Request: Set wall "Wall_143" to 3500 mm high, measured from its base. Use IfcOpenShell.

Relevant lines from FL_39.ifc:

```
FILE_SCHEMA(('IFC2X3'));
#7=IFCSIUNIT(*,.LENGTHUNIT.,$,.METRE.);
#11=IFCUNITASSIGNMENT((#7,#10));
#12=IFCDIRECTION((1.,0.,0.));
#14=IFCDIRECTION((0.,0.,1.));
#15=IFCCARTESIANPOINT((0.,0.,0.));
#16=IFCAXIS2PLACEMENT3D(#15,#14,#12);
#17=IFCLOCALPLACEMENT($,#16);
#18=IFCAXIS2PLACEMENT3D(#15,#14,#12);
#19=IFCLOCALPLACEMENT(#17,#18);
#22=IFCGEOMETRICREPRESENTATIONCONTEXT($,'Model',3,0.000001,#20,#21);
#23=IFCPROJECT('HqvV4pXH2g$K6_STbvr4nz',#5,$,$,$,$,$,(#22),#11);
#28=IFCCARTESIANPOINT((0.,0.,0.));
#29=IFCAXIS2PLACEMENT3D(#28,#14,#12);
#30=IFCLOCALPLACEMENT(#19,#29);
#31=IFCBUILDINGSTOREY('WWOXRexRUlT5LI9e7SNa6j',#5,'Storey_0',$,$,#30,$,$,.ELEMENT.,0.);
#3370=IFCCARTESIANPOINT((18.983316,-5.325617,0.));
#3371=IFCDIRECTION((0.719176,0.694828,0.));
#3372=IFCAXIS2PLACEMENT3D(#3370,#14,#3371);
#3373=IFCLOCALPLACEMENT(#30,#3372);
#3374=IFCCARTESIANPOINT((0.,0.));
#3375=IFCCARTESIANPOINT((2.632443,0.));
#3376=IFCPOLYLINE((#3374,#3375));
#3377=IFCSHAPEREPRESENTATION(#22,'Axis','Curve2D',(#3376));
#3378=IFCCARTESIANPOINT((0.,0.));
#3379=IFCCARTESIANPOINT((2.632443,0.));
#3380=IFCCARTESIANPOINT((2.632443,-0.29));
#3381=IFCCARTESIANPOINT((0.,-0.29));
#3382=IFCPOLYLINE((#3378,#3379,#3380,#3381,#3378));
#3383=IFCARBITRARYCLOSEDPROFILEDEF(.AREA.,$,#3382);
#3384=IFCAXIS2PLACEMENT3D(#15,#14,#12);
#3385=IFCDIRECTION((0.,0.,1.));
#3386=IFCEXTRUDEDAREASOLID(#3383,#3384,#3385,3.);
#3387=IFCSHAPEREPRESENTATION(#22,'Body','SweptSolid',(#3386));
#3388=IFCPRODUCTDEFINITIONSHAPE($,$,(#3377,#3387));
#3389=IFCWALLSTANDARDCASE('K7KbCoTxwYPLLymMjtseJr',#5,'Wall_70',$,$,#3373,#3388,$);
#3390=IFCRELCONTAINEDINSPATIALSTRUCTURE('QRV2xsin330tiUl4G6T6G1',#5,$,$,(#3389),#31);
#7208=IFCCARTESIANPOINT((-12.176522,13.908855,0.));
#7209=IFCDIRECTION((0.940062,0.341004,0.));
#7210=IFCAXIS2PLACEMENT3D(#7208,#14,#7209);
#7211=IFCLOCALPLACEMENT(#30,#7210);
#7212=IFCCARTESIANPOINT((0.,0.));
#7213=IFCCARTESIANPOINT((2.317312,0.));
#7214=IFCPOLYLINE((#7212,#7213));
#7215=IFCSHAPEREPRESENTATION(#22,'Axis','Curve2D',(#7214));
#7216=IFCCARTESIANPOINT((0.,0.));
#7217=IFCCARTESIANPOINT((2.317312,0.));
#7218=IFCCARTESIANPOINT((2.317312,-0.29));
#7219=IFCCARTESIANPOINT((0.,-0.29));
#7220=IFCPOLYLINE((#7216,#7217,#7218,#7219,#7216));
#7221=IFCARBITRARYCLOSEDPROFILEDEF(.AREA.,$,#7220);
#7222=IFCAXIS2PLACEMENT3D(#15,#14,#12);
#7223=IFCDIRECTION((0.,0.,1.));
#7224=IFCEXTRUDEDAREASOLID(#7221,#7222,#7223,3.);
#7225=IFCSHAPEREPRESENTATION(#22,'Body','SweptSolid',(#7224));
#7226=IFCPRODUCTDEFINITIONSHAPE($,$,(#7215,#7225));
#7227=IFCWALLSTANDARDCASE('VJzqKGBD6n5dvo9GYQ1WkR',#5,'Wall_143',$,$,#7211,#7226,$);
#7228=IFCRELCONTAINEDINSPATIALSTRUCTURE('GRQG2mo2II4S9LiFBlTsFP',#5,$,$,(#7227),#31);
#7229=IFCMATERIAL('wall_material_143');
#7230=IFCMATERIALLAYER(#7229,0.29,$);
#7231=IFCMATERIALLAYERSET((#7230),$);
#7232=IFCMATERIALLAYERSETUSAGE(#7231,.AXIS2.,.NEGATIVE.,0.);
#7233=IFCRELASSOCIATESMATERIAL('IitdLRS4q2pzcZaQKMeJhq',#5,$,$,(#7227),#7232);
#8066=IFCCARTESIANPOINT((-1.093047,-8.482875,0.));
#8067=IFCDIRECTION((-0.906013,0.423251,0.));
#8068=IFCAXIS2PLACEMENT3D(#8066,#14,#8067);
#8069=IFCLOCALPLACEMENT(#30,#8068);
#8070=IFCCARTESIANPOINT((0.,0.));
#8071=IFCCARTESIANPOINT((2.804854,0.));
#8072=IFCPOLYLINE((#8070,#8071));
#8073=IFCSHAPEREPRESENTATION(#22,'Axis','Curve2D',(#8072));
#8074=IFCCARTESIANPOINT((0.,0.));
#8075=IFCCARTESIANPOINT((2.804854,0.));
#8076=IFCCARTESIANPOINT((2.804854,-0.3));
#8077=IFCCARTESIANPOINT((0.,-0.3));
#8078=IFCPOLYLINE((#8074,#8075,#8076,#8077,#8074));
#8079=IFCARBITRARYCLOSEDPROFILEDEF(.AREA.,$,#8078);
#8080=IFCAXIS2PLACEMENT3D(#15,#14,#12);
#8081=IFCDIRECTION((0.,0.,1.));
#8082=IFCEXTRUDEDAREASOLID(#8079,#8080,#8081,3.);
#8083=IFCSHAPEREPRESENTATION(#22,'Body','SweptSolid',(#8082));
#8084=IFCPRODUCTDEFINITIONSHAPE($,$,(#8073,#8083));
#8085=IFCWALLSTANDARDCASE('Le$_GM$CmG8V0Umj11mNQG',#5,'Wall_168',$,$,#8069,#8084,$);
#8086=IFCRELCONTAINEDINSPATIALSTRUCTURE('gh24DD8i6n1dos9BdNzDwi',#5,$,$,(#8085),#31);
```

```python
import ifcopenshell
import ifcopenshell.geom
import ifcopenshell.util.shape

model = ifcopenshell.open("FL_39.ifc")
settings = ifcopenshell.geom.settings()


def volume(element):
    """Net volume in cubic metres, openings subtracted."""
    shape = ifcopenshell.geom.create_shape(settings, element)
    return ifcopenshell.util.shape.get_volume(shape.geometry)


wall = model.by_id(7227)
before = volume(wall)

body = next(r for r in wall.Representation.Representations if r.RepresentationIdentifier == "Body")
solid = body.Items[0]
old_height = solid.Depth
solid.Depth = 3.5
after = volume(wall)

print(f"height {old_height:g} -> {solid.Depth:g}, volume {before:.3f} -> {after:.3f} m3")

model.write("FL_39_rev.ifc")
```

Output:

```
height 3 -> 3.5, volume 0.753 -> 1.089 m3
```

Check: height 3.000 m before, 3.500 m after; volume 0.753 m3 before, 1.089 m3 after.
